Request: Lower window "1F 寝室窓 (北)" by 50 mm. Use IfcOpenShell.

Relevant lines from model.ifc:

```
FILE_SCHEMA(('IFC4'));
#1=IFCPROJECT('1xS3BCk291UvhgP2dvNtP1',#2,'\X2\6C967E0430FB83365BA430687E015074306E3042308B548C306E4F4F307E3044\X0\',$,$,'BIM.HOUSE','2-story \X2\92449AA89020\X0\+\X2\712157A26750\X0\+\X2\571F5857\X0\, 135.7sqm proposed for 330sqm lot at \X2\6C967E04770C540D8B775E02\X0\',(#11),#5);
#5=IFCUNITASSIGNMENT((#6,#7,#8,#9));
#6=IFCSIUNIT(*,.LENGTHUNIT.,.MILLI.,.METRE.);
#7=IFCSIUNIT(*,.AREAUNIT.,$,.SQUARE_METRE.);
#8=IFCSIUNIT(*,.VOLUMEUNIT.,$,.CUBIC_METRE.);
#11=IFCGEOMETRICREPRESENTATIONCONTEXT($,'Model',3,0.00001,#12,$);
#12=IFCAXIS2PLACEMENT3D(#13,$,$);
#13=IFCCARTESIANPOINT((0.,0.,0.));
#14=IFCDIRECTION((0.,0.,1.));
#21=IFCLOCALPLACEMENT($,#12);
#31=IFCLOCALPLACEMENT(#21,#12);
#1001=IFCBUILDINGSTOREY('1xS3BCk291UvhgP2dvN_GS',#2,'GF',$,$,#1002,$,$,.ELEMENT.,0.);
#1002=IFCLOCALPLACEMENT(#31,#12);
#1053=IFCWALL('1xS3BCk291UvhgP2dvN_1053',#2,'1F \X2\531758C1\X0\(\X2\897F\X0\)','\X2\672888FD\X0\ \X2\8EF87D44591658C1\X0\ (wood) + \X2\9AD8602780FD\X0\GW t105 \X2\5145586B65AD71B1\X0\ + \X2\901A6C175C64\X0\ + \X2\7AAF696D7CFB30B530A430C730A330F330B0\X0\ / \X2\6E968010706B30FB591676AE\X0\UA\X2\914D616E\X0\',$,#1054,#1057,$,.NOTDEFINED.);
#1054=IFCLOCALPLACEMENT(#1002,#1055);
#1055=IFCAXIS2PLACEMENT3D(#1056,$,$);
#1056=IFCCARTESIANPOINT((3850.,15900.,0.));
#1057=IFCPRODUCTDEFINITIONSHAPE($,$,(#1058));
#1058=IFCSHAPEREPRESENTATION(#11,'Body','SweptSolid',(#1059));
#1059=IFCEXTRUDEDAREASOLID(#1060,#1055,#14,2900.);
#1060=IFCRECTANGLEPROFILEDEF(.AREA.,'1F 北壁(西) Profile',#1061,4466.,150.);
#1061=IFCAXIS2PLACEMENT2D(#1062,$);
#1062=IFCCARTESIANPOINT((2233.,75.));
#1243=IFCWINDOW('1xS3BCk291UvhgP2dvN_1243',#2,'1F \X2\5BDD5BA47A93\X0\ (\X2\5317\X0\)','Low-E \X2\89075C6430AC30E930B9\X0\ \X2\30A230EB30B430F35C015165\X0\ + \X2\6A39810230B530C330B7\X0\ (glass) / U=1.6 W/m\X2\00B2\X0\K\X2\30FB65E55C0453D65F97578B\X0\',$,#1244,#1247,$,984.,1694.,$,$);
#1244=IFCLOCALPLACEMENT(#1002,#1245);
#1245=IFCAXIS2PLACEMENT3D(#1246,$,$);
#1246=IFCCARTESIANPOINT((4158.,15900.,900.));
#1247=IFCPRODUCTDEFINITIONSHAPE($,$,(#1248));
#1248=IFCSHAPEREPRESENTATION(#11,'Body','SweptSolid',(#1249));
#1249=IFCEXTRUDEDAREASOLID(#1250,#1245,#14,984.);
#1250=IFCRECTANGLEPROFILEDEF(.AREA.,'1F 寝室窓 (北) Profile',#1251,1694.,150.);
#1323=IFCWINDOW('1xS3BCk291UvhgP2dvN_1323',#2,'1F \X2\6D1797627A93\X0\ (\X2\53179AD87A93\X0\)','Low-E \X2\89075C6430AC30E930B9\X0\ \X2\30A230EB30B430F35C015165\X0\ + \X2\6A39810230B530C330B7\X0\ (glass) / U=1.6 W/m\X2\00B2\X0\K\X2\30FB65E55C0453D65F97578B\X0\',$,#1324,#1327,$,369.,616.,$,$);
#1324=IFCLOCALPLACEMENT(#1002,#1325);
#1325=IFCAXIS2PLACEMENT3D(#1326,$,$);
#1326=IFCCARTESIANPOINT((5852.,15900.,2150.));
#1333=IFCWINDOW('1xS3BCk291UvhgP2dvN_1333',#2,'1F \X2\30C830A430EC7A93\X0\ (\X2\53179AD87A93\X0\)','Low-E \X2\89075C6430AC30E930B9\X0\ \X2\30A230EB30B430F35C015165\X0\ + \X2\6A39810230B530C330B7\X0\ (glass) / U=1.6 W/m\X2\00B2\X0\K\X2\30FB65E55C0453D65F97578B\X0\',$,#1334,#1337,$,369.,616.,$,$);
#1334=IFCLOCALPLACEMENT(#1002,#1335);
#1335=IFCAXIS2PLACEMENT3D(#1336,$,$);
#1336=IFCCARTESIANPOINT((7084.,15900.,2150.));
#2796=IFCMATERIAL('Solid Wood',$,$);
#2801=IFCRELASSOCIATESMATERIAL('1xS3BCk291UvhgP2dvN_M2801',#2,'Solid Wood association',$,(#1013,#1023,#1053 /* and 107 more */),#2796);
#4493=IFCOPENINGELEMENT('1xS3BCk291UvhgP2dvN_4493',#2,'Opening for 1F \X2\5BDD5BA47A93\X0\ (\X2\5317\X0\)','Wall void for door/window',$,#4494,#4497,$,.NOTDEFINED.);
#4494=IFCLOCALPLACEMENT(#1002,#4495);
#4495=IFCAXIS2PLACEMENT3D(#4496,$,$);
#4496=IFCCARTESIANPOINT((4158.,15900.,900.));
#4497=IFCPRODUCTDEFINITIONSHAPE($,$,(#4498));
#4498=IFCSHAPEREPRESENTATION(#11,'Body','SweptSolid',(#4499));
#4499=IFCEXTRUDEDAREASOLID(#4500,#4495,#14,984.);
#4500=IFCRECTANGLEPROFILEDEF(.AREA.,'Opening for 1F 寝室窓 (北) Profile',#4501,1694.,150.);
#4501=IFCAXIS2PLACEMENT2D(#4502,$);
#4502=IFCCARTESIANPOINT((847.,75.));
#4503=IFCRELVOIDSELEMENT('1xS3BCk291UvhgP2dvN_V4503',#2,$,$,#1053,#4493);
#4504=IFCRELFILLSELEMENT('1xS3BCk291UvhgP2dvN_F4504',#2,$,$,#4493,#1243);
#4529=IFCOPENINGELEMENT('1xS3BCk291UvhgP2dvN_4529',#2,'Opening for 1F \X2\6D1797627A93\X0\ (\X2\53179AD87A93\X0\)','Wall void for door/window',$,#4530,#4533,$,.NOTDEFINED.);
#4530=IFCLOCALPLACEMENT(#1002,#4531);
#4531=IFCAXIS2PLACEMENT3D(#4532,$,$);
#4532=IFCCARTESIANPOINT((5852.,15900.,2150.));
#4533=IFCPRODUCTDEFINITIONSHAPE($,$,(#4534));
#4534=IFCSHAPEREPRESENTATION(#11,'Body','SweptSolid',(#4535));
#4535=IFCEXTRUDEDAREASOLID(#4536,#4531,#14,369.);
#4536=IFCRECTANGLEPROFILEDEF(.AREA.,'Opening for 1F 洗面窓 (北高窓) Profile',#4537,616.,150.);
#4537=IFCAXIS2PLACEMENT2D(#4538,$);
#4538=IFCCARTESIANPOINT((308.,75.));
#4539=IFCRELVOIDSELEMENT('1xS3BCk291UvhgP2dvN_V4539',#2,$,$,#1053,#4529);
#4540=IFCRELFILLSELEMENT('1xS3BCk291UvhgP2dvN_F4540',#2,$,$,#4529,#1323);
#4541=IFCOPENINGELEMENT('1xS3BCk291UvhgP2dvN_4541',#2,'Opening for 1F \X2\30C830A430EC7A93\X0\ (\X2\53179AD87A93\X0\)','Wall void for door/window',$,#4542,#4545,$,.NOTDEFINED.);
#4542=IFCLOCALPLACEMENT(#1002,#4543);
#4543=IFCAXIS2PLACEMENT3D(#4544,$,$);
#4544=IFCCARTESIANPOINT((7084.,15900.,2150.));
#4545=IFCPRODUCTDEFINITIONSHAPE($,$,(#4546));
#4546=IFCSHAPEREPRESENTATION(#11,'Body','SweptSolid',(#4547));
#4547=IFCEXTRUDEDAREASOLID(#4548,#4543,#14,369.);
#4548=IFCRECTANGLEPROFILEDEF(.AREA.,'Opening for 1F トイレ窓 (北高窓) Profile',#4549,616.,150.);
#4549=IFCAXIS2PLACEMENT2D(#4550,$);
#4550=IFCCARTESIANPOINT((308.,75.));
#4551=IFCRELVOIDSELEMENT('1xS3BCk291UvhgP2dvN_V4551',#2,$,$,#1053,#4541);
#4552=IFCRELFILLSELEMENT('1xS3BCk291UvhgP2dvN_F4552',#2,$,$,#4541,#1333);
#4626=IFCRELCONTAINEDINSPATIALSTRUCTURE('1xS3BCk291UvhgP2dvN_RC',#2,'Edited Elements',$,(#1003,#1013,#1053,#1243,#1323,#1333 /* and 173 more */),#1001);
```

```python
import numpy as np
import ifcopenshell
import ifcopenshell.api.geometry
import ifcopenshell.util.placement
import ifcopenshell.util.unit

model = ifcopenshell.open("model.ifc")
unit_scale = ifcopenshell.util.unit.calculate_unit_scale(model)

window = model.by_guid("1xS3BCk291UvhgP2dvN_1243")
opening = window.FillsVoids[0].RelatingOpeningElement
dz = -50.0

shift = np.array([0.0, 0.0, dz])
# The window is not placed relative to its opening, so move both.
for product in (opening, window):
    matrix = ifcopenshell.util.placement.get_local_placement(product.ObjectPlacement)
    matrix[:3, 3] += shift
    ifcopenshell.api.geometry.edit_object_placement(model, product=product, matrix=matrix, is_si=False)

print(f"moved by {dz * unit_scale:+.3f} m")

model.write("model_v2.ifc")
```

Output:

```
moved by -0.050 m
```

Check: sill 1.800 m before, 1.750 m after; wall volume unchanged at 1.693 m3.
